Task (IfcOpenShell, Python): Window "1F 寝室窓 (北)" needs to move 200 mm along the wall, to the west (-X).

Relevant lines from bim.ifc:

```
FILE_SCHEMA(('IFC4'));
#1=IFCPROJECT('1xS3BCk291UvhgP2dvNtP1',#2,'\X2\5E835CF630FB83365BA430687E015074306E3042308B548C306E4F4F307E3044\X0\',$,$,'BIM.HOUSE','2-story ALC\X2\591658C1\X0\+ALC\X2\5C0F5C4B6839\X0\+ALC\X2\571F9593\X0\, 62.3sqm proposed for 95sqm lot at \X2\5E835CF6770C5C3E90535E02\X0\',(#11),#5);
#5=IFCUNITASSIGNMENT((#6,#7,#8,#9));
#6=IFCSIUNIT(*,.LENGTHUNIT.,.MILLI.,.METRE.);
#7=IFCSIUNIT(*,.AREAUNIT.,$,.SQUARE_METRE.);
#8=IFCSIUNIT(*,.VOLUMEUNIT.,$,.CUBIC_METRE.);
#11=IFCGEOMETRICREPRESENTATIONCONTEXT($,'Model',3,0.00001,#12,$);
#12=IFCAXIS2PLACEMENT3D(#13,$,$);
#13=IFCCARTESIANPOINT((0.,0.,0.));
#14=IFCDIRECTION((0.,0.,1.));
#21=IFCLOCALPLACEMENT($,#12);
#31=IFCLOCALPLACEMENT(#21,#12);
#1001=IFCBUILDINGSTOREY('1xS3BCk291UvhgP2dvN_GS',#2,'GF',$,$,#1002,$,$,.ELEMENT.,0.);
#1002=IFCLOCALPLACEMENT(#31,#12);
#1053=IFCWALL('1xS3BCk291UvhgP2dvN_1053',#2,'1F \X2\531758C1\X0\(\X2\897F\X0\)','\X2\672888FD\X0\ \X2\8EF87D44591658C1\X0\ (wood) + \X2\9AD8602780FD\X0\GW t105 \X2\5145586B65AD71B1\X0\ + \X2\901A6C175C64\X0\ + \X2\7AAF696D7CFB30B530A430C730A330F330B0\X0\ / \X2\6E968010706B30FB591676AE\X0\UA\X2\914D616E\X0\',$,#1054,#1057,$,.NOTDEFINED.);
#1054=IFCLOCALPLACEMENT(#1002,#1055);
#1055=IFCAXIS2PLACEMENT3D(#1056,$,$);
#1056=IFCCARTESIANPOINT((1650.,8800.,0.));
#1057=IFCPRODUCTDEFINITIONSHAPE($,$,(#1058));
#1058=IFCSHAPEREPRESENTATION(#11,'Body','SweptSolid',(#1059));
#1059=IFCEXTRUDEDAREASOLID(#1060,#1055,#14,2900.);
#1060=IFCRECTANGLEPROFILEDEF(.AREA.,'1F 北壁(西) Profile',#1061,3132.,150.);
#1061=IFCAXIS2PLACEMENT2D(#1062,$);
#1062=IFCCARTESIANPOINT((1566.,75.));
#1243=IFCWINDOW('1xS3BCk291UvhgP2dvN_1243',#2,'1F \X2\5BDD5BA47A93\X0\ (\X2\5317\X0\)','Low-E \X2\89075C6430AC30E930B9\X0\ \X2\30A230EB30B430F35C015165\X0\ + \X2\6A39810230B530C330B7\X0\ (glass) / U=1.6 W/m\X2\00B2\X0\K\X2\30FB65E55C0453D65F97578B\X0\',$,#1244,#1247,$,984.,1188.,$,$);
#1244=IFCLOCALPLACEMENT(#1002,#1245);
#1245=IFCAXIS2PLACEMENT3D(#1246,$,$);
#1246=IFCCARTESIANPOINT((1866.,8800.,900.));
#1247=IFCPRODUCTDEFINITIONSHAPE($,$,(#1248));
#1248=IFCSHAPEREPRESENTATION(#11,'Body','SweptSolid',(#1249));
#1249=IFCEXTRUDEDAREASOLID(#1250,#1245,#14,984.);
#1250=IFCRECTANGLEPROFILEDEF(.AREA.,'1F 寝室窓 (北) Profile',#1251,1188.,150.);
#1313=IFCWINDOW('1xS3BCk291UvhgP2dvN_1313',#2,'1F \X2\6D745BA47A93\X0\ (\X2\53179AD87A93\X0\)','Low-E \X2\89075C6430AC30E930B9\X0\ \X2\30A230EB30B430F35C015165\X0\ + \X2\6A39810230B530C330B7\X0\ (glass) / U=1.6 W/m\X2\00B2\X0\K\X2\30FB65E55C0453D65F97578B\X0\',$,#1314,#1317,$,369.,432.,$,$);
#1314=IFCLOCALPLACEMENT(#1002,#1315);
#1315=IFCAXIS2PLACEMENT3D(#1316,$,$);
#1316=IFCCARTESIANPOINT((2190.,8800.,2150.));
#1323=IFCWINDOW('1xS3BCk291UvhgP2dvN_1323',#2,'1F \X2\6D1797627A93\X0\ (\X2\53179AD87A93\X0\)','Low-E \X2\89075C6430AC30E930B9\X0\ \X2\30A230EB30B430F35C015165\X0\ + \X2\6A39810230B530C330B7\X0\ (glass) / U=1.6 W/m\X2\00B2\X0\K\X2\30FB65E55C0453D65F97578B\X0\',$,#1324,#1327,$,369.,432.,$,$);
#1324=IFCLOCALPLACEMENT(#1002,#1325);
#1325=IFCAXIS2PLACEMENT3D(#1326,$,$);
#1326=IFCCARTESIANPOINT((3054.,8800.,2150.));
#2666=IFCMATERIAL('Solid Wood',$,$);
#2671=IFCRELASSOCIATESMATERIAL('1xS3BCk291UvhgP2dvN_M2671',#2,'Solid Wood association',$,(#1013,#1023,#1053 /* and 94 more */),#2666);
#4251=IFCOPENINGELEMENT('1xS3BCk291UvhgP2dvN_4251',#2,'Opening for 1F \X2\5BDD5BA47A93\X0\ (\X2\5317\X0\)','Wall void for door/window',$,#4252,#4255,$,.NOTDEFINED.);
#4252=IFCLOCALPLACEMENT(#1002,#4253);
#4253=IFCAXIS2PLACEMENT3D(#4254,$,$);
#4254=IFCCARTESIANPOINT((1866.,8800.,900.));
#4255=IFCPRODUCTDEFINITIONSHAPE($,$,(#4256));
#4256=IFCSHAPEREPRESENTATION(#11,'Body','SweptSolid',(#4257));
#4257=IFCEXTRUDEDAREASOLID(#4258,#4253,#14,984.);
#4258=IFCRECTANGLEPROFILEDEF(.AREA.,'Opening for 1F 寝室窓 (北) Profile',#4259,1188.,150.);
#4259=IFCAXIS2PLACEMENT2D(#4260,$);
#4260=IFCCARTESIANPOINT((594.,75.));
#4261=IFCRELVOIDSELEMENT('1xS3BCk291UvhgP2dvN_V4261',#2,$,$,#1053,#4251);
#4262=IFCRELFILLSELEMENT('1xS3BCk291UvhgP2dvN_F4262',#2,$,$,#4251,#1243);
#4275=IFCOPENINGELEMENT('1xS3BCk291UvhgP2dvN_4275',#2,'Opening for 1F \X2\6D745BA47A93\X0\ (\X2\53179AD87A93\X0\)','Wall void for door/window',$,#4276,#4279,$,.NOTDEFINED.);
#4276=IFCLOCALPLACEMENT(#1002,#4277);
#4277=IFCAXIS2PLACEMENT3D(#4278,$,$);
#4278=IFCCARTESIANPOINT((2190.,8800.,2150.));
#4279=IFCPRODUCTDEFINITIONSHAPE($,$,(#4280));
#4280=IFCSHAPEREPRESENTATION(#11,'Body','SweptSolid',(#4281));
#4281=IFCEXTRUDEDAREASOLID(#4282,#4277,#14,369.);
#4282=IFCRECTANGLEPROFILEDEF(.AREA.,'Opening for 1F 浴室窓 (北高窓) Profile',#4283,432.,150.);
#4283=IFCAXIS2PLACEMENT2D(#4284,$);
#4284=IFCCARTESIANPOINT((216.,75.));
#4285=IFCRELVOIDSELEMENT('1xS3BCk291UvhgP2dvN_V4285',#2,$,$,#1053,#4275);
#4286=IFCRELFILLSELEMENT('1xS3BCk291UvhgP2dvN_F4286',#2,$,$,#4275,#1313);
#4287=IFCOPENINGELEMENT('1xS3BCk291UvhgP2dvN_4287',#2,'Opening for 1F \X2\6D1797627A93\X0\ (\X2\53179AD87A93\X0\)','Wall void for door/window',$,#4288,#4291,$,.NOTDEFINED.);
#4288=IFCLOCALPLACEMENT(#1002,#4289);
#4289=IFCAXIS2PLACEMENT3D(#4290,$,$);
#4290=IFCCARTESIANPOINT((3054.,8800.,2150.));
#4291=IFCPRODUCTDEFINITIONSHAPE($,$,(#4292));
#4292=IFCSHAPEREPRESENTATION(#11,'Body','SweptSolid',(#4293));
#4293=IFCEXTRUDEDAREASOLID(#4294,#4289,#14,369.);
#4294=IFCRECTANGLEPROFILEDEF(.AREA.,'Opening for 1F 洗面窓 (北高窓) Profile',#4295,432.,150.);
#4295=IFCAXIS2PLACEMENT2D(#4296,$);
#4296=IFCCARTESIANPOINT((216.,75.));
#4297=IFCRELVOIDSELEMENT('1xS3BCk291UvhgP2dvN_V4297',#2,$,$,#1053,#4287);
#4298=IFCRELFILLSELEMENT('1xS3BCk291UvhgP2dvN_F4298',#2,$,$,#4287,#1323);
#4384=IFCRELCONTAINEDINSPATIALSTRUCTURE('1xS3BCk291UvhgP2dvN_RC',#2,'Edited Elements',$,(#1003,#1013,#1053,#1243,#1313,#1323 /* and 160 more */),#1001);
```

```python
import ifcopenshell
import ifcopenshell.api.geometry
import ifcopenshell.util.placement
import ifcopenshell.util.unit

model = ifcopenshell.open("bim.ifc")
unit_scale = ifcopenshell.util.unit.calculate_unit_scale(model)

window = model.by_guid("1xS3BCk291UvhgP2dvN_1243")
opening = window.FillsVoids[0].RelatingOpeningElement
wall = opening.VoidsElements[0].RelatingBuildingElement

wall_matrix = ifcopenshell.util.placement.get_local_placement(wall.ObjectPlacement)
shift = wall_matrix[:3, 0] * -0.2 / unit_scale
before = ifcopenshell.util.placement.get_local_placement(window.ObjectPlacement)[:3, 3].copy()

# The window is not placed relative to its opening, so move both.
for product in (opening, window):
    matrix = ifcopenshell.util.placement.get_local_placement(product.ObjectPlacement)
    matrix[:3, 3] += shift
    ifcopenshell.api.geometry.edit_object_placement(model, product=product, matrix=matrix, is_si=False)

after = ifcopenshell.util.placement.get_local_placement(window.ObjectPlacement)[:3, 3]
print("window moved by", (after - before).round(3) + 0.0)

model.write("bim_updated.ifc")
```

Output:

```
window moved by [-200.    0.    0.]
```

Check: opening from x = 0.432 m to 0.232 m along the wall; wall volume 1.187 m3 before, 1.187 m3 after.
